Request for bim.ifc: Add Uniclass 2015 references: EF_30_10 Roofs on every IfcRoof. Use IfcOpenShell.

First a look at what the model holds.

```python
import ifcopenshell

model = ifcopenshell.open("bim.ifc")
print(model.schema)
print("classifications:", [c.Name for c in model.by_type("IfcClassification")])
for ifc_class in ("IfcDoor", "IfcRoof", "IfcStair", "IfcWall", "IfcWindow"):
    print(ifc_class, len(model.by_type(ifc_class)))
```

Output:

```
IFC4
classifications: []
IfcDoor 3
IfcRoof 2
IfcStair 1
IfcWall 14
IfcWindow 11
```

```python
import ifcopenshell
import ifcopenshell.api.classification

model = ifcopenshell.open("bim.ifc")

system = ifcopenshell.api.classification.add_classification(model, classification="Uniclass 2015")

codes = {
    "IfcRoof": ("EF_30_10", "Roofs"),
}
for ifc_class, (code, name) in codes.items():
    products = model.by_type(ifc_class)
    ifcopenshell.api.classification.add_reference(
        model, products=products, classification=system, identification=code, name=name
    )
    print(code, len(products))

model.write("bim_v2.ifc")
```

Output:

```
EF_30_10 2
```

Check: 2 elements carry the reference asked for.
